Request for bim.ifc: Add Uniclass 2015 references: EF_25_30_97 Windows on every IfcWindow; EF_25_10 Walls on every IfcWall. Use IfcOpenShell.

First a look at what the model holds.

```python
import ifcopenshell

model = ifcopenshell.open("bim.ifc")
print(model.schema)
print("classifications:", [c.Name for c in model.by_type("IfcClassification")])
for ifc_class in ("IfcDoor", "IfcRoof", "IfcStair", "IfcWall", "IfcWindow"):
    print(ifc_class, len(model.by_type(ifc_class)))
```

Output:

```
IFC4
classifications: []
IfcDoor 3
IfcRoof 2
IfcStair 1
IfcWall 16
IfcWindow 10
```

```python
import ifcopenshell
import ifcopenshell.api.classification

model = ifcopenshell.open("bim.ifc")

system = ifcopenshell.api.classification.add_classification(model, classification="Uniclass 2015")

codes = {
    "IfcWindow": ("EF_25_30_97", "Windows"),
    "IfcWall": ("EF_25_10", "Walls"),
}
for ifc_class, (code, name) in codes.items():
    products = model.by_type(ifc_class)
    ifcopenshell.api.classification.add_reference(
        model, products=products, classification=system, identification=code, name=name
    )
    print(code, len(products))

model.write("bim_rev.ifc")
```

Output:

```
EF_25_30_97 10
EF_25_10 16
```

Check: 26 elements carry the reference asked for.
